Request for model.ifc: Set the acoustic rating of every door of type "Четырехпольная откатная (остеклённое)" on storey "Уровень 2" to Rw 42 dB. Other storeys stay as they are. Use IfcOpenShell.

First a look at what the model holds.

```python
import ifcopenshell
import ifcopenshell.util.element

model = ifcopenshell.open("model.ifc")
print(model.schema)
storey = next(s for s in model.by_type("IfcBuildingStorey") if s.Name == "Уровень 2")
doors = [e for e in ifcopenshell.util.element.get_decomposition(storey) if e.is_a("IfcDoor")]
seen = {}
for e in doors:
    element_type = ifcopenshell.util.element.get_type(e)
    key = (element_type.Name if element_type != e and element_type else None, ifcopenshell.util.element.get_pset(e, "Pset_DoorCommon", "AcousticRating"))
    seen[key] = seen.get(key, 0) + 1
for (name, value), count in sorted(seen.items(), key=str):
    print(count, "x", name, "|", value)
```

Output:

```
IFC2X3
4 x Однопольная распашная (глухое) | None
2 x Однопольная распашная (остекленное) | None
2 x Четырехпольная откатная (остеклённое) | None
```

```python
import ifcopenshell
import ifcopenshell.api.pset
import ifcopenshell.util.element

model = ifcopenshell.open("model.ifc")

storey = next(s for s in model.by_type("IfcBuildingStorey") if s.Name == "Уровень 2")
doors = [e for e in ifcopenshell.util.element.get_decomposition(storey) if e.is_a("IfcDoor")]

count = 0
for e in doors:
    element_type = ifcopenshell.util.element.get_type(e)
    if element_type in (None, e) or element_type.Name != "Четырехпольная откатная (остеклённое)":
        continue
    # add_pset returns the element's existing set when there is one.
    pset = ifcopenshell.api.pset.add_pset(model, product=e, name="Pset_DoorCommon")
    ifcopenshell.api.pset.edit_pset(model, pset=pset, properties={"AcousticRating": "Rw 42 dB"})
    count += 1

print(count, "doors updated")

model.write("model-out.ifc")
```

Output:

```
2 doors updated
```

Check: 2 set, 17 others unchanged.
